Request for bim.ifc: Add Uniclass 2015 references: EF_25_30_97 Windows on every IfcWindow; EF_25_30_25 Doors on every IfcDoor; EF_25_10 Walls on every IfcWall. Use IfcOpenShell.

First a look at what the model holds.

```python
import ifcopenshell

model = ifcopenshell.open("bim.ifc")
print(model.schema)
print("classifications:", [c.Name for c in model.by_type("IfcClassification")])
for ifc_class in ("IfcDoor", "IfcRoof", "IfcStair", "IfcWall", "IfcWindow"):
    print(ifc_class, len(model.by_type(ifc_class)))
```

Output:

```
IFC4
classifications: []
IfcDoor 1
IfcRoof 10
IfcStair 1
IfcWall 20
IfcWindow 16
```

```python
import ifcopenshell
import ifcopenshell.api.classification

model = ifcopenshell.open("bim.ifc")

system = ifcopenshell.api.classification.add_classification(model, classification="Uniclass 2015")

codes = {
    "IfcWindow": ("EF_25_30_97", "Windows"),
    "IfcDoor": ("EF_25_30_25", "Doors"),
    "IfcWall": ("EF_25_10", "Walls"),
}
for ifc_class, (code, name) in codes.items():
    products = model.by_type(ifc_class)
    ifcopenshell.api.classification.add_reference(
        model, products=products, classification=system, identification=code, name=name
    )
    print(code, len(products))

model.write("bim_v2.ifc")
```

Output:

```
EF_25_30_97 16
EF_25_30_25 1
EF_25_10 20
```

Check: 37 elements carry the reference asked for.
